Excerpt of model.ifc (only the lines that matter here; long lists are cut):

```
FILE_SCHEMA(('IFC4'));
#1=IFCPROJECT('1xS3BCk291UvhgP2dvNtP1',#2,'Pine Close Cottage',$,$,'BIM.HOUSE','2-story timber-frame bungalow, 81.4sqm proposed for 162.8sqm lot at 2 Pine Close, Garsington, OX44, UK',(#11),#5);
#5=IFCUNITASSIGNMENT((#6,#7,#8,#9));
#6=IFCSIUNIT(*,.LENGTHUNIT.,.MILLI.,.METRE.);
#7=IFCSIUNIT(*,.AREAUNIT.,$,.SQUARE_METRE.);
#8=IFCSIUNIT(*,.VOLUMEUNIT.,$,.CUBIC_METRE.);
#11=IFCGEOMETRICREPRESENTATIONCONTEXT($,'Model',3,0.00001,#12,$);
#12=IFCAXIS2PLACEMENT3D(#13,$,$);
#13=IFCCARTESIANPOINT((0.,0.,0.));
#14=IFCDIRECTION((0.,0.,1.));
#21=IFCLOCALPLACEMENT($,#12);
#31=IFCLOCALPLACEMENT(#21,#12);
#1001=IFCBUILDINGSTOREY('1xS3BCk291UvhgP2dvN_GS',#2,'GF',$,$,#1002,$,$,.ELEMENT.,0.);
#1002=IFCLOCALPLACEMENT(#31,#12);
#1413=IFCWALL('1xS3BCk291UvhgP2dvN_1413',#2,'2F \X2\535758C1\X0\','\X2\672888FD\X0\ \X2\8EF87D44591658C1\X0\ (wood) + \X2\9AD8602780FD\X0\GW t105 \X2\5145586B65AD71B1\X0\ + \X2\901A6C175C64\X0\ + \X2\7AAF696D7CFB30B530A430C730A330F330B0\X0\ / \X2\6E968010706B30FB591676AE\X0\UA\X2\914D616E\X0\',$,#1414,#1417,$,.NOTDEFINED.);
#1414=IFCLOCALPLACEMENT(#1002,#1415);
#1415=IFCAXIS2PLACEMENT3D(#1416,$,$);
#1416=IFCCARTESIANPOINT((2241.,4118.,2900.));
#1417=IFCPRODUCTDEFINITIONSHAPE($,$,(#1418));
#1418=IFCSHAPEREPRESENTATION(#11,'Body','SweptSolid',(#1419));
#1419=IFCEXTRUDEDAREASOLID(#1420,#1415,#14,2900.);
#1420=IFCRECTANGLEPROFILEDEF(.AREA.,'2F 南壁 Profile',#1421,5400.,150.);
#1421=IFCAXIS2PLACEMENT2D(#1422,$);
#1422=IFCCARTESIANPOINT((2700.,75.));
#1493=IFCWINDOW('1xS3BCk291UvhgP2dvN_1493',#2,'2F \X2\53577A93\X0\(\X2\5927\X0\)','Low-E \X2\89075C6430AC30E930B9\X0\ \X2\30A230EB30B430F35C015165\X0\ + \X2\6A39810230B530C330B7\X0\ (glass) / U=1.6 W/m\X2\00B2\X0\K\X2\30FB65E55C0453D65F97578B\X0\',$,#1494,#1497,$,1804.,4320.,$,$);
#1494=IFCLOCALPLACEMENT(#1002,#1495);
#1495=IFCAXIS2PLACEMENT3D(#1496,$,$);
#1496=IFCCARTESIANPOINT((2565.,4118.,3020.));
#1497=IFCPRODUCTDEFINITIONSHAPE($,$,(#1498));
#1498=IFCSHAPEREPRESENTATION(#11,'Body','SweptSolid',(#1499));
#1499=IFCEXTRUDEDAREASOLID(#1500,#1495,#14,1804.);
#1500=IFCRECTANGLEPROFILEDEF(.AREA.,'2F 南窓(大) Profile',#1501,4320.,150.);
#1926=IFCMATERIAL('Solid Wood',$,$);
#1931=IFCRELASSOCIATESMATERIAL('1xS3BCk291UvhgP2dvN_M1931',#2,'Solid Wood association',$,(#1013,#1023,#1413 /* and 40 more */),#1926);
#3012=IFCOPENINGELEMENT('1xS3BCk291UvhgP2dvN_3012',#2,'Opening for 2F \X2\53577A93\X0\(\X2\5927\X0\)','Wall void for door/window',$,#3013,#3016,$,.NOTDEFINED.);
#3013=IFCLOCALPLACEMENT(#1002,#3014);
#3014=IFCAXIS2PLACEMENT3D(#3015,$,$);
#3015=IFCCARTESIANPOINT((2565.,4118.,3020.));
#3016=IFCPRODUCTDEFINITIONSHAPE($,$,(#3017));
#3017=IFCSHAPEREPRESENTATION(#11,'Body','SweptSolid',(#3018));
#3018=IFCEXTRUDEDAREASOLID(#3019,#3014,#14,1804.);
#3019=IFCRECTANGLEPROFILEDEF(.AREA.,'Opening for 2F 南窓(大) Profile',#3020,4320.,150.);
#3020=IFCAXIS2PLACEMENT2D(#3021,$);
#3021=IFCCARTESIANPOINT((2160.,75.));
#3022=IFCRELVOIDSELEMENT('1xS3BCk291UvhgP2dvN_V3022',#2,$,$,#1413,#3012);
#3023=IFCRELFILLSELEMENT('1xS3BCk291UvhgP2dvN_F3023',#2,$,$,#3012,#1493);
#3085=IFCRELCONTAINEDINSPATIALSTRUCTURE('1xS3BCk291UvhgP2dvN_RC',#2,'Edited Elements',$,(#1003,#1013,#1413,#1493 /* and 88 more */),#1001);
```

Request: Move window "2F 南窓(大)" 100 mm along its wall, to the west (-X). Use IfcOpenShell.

```python
import ifcopenshell
import ifcopenshell.api.geometry
import ifcopenshell.util.placement
import ifcopenshell.util.unit

model = ifcopenshell.open("model.ifc")
unit_scale = ifcopenshell.util.unit.calculate_unit_scale(model)

window = model.by_guid("1xS3BCk291UvhgP2dvN_1493")
opening = window.FillsVoids[0].RelatingOpeningElement
wall = opening.VoidsElements[0].RelatingBuildingElement

wall_matrix = ifcopenshell.util.placement.get_local_placement(wall.ObjectPlacement)
shift = wall_matrix[:3, 0] * -0.1 / unit_scale
before = ifcopenshell.util.placement.get_local_placement(window.ObjectPlacement)[:3, 3].copy()

# The window is not placed relative to its opening, so move both.
for product in (opening, window):
    matrix = ifcopenshell.util.placement.get_local_placement(product.ObjectPlacement)
    matrix[:3, 3] += shift
    ifcopenshell.api.geometry.edit_object_placement(model, product=product, matrix=matrix, is_si=False)

after = ifcopenshell.util.placement.get_local_placement(window.ObjectPlacement)[:3, 3]
print("window moved by", (after - before).round(3) + 0.0)

model.write("model_updated.ifc")
```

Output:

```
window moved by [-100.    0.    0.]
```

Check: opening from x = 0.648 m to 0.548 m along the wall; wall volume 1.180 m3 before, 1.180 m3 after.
